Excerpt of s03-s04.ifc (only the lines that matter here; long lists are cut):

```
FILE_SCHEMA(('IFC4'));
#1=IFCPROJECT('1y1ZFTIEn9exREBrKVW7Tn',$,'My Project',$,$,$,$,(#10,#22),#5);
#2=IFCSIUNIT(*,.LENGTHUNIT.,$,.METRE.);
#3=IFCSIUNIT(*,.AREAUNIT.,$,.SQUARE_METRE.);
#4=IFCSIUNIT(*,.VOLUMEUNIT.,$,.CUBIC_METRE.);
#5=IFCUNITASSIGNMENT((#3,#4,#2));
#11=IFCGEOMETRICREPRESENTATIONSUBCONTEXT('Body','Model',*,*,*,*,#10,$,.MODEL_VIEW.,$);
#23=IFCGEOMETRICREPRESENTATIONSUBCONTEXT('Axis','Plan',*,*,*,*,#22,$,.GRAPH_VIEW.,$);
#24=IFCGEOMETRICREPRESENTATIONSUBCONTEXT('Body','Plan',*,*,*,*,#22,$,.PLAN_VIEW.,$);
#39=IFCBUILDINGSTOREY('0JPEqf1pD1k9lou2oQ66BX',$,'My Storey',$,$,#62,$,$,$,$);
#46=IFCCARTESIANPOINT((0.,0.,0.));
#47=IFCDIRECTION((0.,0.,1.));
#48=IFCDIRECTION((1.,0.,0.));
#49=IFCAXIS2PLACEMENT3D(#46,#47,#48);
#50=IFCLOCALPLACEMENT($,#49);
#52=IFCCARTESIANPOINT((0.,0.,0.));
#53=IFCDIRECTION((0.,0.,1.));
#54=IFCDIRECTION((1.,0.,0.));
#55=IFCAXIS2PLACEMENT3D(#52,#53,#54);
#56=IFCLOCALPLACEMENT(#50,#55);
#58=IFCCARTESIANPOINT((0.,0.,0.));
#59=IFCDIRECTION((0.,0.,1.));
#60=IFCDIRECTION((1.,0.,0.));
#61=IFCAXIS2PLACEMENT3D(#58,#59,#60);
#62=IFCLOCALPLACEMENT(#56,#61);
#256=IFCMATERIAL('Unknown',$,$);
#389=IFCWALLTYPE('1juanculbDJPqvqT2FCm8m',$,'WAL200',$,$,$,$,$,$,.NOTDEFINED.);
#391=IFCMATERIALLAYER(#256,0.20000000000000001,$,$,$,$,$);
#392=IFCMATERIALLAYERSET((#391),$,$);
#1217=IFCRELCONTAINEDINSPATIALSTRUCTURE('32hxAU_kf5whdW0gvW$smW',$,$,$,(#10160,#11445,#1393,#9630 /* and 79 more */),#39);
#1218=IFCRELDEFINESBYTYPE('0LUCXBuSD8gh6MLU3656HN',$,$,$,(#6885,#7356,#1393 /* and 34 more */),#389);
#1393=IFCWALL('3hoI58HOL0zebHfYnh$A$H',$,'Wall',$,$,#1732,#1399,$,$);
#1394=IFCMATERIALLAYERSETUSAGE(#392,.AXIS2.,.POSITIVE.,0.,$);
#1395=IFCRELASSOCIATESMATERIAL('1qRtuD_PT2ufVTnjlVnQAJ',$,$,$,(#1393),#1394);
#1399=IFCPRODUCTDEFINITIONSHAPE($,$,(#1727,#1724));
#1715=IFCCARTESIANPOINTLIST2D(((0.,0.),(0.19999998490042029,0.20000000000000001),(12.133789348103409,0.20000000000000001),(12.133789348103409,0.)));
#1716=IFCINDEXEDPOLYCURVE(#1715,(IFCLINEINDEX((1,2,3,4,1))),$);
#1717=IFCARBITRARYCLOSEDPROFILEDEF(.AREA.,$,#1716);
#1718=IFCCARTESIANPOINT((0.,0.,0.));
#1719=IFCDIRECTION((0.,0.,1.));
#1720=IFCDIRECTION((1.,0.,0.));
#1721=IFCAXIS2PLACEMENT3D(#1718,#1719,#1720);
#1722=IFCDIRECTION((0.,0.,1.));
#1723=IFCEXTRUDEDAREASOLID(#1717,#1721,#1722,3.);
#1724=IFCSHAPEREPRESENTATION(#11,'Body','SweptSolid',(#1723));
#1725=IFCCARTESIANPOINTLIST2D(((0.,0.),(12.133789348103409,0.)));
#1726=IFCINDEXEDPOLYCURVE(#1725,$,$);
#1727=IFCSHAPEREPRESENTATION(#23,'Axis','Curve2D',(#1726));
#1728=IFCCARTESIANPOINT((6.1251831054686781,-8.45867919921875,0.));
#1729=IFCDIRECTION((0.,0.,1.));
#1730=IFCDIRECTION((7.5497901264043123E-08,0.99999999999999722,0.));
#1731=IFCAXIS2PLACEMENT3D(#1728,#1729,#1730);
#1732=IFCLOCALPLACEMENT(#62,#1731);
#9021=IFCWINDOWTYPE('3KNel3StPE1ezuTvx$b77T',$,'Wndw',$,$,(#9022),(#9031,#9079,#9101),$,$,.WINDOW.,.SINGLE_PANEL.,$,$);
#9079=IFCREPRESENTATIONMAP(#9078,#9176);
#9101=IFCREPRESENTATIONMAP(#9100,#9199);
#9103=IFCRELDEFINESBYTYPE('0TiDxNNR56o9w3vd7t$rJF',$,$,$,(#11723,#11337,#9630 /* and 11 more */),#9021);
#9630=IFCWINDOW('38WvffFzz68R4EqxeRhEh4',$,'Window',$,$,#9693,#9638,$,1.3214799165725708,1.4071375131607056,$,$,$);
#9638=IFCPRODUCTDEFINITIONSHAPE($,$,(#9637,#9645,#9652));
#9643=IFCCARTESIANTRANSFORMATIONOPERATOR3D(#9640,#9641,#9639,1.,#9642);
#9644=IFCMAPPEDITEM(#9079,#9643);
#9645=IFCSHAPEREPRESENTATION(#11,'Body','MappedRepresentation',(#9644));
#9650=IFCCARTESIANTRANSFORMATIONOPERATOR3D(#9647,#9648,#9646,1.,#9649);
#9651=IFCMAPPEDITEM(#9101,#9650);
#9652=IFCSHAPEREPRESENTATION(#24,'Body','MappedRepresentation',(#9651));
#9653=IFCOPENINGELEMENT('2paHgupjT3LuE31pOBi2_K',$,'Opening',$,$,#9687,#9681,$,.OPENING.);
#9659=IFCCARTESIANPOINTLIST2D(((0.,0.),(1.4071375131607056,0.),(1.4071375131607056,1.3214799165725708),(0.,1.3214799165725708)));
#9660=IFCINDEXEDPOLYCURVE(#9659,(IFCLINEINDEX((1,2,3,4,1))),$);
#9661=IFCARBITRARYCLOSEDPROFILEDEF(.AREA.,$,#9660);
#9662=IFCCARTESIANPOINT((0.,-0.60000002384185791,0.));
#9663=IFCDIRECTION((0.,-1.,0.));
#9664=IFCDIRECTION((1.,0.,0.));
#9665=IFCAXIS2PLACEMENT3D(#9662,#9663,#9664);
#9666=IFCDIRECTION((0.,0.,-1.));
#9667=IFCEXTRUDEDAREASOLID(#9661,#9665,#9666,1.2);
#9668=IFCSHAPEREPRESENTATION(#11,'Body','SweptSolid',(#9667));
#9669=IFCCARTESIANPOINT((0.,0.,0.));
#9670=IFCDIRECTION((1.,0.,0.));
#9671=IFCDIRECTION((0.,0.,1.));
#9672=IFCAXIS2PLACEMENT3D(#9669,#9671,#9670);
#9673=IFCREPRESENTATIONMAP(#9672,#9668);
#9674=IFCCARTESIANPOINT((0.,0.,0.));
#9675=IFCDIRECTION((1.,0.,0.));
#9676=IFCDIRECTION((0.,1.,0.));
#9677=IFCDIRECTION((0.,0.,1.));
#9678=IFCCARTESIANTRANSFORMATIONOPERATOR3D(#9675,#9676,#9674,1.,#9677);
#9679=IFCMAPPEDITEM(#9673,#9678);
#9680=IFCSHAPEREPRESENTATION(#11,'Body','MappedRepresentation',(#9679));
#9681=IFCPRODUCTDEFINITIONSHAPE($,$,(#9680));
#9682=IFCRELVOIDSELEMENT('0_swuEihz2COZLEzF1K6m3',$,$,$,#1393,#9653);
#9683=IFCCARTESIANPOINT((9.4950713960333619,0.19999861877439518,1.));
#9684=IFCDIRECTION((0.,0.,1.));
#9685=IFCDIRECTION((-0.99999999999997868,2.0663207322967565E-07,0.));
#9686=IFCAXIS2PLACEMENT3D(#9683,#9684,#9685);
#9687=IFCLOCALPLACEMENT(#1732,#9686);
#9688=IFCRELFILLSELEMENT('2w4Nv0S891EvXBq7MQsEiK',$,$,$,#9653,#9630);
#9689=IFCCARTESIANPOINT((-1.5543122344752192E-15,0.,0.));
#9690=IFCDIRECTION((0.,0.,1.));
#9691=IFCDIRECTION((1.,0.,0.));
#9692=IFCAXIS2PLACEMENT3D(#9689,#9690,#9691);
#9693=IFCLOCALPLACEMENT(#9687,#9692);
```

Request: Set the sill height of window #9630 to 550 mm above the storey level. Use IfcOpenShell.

```python
import numpy as np
import ifcopenshell
import ifcopenshell.api.geometry
import ifcopenshell.geom
import ifcopenshell.util.element
import ifcopenshell.util.placement
import ifcopenshell.util.shape
import ifcopenshell.util.unit

model = ifcopenshell.open("s03-s04.ifc")
unit_scale = ifcopenshell.util.unit.calculate_unit_scale(model)

window = model.by_id(9630)
opening = window.FillsVoids[0].RelatingOpeningElement
storey = ifcopenshell.util.element.get_container(window, ifc_class="IfcBuildingStorey")
level = ifcopenshell.util.placement.get_local_placement(storey.ObjectPlacement)[2, 3]

# The opening's origin need not be at the sill, so measure its lowest point.
shape = ifcopenshell.geom.create_shape(ifcopenshell.geom.settings(), opening)
bottom = ifcopenshell.util.shape.get_shape_bottom_elevation(shape, shape.geometry) / unit_scale
dz = level + 0.55 / unit_scale - bottom

shift = np.array([0.0, 0.0, dz])
# The window is placed relative to its opening, so it follows when the opening moves.
matrix = ifcopenshell.util.placement.get_local_placement(opening.ObjectPlacement)
matrix[:3, 3] += shift
ifcopenshell.api.geometry.edit_object_placement(
    model, product=opening, matrix=matrix, is_si=False, should_transform_children=True
)

print(f"moved by {dz * unit_scale:+.3f} m")

model.write("s03-s04_edited.ifc")
```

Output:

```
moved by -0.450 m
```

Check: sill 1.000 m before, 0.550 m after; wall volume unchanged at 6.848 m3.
